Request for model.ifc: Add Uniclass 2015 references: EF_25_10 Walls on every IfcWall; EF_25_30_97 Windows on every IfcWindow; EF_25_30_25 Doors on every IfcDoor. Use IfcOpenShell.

First a look at what the model holds.

```python
import ifcopenshell

model = ifcopenshell.open("model.ifc")
print(model.schema)
print("classifications:", [c.Name for c in model.by_type("IfcClassification")])
for ifc_class in ("IfcDoor", "IfcRoof", "IfcStair", "IfcWall", "IfcWindow"):
    print(ifc_class, len(model.by_type(ifc_class)))
```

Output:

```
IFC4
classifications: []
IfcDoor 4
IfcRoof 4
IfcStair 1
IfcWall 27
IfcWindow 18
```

```python
import ifcopenshell
import ifcopenshell.api.classification

model = ifcopenshell.open("model.ifc")

system = ifcopenshell.api.classification.add_classification(model, classification="Uniclass 2015")

codes = {
    "IfcWall": ("EF_25_10", "Walls"),
    "IfcWindow": ("EF_25_30_97", "Windows"),
    "IfcDoor": ("EF_25_30_25", "Doors"),
}
for ifc_class, (code, name) in codes.items():
    products = model.by_type(ifc_class)
    ifcopenshell.api.classification.add_reference(
        model, products=products, classification=system, identification=code, name=name
    )
    print(code, len(products))

model.write("model_rev.ifc")
```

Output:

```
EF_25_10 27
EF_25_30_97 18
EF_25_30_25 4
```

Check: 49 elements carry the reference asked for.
